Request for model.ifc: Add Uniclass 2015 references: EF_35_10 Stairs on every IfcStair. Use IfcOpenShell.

First a look at what the model holds.

```python
import ifcopenshell

model = ifcopenshell.open("model.ifc")
print(model.schema)
print("classifications:", [c.Name for c in model.by_type("IfcClassification")])
for ifc_class in ("IfcDoor", "IfcRoof", "IfcStair", "IfcWall", "IfcWindow"):
    print(ifc_class, len(model.by_type(ifc_class)))
```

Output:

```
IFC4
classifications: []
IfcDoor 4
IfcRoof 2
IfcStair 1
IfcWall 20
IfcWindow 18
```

```python
import ifcopenshell
import ifcopenshell.api.classification

model = ifcopenshell.open("model.ifc")

system = ifcopenshell.api.classification.add_classification(model, classification="Uniclass 2015")

codes = {
    "IfcStair": ("EF_35_10", "Stairs"),
}
for ifc_class, (code, name) in codes.items():
    products = model.by_type(ifc_class)
    ifcopenshell.api.classification.add_reference(
        model, products=products, classification=system, identification=code, name=name
    )
    print(code, len(products))

model.write("model_updated.ifc")
```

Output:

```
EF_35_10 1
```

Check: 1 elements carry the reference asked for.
